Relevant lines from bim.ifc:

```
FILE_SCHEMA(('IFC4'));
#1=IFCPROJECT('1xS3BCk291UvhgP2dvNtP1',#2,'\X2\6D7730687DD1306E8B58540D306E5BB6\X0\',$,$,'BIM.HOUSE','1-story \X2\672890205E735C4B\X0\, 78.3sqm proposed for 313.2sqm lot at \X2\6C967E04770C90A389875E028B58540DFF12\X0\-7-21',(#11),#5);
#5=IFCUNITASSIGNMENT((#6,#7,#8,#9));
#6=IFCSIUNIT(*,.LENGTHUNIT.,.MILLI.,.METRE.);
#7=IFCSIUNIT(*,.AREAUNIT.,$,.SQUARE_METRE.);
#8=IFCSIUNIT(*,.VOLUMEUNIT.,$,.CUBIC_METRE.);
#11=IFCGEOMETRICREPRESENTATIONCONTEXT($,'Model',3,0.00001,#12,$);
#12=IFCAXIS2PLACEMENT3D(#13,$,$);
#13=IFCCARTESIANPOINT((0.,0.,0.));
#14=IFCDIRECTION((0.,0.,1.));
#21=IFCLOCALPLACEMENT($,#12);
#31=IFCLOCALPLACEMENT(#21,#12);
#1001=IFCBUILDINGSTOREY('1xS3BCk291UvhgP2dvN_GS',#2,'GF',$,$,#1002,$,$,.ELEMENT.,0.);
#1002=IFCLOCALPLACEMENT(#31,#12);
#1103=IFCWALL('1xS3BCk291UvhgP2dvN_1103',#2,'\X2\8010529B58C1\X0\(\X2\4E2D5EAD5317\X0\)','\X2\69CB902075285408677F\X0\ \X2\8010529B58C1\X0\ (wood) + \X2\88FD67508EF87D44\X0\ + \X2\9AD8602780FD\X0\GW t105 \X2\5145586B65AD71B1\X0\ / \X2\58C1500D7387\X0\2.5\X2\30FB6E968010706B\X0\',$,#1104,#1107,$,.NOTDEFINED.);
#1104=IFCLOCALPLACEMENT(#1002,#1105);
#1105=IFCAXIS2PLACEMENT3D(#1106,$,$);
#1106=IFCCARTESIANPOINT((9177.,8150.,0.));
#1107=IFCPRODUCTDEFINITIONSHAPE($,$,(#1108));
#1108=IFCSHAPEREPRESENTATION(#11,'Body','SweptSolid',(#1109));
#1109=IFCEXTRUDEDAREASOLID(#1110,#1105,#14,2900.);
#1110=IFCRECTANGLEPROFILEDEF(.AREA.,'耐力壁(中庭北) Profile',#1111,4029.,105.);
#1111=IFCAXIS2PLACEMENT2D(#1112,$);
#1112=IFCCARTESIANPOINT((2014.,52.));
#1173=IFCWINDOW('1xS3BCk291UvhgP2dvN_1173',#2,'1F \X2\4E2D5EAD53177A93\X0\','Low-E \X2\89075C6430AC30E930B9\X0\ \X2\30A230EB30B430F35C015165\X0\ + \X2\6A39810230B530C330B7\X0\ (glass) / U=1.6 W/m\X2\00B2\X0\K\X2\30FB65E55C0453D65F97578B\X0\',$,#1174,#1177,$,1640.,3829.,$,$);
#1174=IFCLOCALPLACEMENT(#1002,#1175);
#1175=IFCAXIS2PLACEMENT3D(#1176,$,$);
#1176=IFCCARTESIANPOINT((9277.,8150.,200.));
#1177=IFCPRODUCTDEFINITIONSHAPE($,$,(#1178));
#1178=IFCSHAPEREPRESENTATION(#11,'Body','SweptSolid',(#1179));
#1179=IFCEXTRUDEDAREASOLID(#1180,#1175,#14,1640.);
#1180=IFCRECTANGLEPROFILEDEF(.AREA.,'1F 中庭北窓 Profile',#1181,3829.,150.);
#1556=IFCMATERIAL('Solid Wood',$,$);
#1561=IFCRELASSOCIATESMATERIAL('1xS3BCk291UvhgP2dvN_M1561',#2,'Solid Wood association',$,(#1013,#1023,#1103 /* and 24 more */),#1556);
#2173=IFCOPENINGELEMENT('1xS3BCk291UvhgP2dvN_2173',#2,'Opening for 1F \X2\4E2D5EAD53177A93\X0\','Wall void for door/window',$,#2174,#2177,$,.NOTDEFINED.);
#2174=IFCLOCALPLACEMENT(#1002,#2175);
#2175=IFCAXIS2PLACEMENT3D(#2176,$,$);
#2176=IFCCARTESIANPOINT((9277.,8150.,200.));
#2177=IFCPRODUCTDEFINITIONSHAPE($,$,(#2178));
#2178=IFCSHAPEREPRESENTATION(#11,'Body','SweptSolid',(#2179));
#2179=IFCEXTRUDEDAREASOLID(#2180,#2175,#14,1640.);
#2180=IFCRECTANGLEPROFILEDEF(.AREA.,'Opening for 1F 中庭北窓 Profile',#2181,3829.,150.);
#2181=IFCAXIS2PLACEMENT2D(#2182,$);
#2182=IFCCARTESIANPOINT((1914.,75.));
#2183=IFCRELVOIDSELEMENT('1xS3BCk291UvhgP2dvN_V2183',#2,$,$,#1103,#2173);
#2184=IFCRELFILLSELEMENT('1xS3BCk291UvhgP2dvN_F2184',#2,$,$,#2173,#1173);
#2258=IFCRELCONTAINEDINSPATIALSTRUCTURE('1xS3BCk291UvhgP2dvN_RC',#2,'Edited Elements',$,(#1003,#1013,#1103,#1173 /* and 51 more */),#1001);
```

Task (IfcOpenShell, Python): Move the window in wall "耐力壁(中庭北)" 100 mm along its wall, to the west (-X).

```python
import ifcopenshell
import ifcopenshell.api.geometry
import ifcopenshell.util.placement

model = ifcopenshell.open("bim.ifc")

window = model.by_guid("1xS3BCk291UvhgP2dvN_1173")
opening = window.FillsVoids[0].RelatingOpeningElement
wall = opening.VoidsElements[0].RelatingBuildingElement

wall_matrix = ifcopenshell.util.placement.get_local_placement(wall.ObjectPlacement)
shift = wall_matrix[:3, 0] * -100.0
before = ifcopenshell.util.placement.get_local_placement(window.ObjectPlacement)[:3, 3].copy()

# The window is not placed relative to its opening, so move both.
for product in (opening, window):
    matrix = ifcopenshell.util.placement.get_local_placement(product.ObjectPlacement)
    matrix[:3, 3] += shift
    ifcopenshell.api.geometry.edit_object_placement(model, product=product, matrix=matrix, is_si=False)

after = ifcopenshell.util.placement.get_local_placement(window.ObjectPlacement)[:3, 3]
print("window moved by", (after - before).round(3) + 0.0)

model.write("bim_v2.ifc")
```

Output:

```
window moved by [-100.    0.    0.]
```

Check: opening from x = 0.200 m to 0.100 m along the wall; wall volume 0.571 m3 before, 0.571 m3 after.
